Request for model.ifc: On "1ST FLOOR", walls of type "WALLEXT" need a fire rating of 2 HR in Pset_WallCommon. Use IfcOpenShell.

First a look at what the model holds.

```python
import ifcopenshell
import ifcopenshell.util.element

model = ifcopenshell.open("model.ifc")
print(model.schema)
storey = next(s for s in model.by_type("IfcBuildingStorey") if s.Name == "1ST FLOOR")
walls = [e for e in ifcopenshell.util.element.get_decomposition(storey) if e.is_a("IfcWall")]
seen = {}
for e in walls:
    element_type = ifcopenshell.util.element.get_type(e)
    key = (element_type.Name if element_type != e and element_type else None, ifcopenshell.util.element.get_pset(e, "Pset_WallCommon", "FireRating"))
    seen[key] = seen.get(key, 0) + 1
for (name, value), count in sorted(seen.items(), key=str):
    print(count, "x", name, "|", value)
```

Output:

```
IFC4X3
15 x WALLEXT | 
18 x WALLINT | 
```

```python
import ifcopenshell
import ifcopenshell.api.pset
import ifcopenshell.util.element

model = ifcopenshell.open("model.ifc")

storey = next(s for s in model.by_type("IfcBuildingStorey") if s.Name == "1ST FLOOR")
walls = [e for e in ifcopenshell.util.element.get_decomposition(storey) if e.is_a("IfcWall")]

count = 0
for e in walls:
    element_type = ifcopenshell.util.element.get_type(e)
    if element_type in (None, e) or element_type.Name != "WALLEXT":
        continue
    # add_pset returns the element's existing set when there is one.
    pset = ifcopenshell.api.pset.add_pset(model, product=e, name="Pset_WallCommon")
    ifcopenshell.api.pset.edit_pset(model, pset=pset, properties={"FireRating": "2 HR"})
    count += 1

print(count, "walls updated")

model.write("model_edited.ifc")
```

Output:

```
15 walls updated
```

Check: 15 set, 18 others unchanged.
